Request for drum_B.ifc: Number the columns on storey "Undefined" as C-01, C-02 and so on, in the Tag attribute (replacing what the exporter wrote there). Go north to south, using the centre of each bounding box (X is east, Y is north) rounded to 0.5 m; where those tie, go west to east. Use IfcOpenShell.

First a look at what the model holds.

```python
import ifcopenshell
import ifcopenshell.util.element
import ifcopenshell.util.placement

model = ifcopenshell.open("drum_B.ifc")
print(model.schema)
storey = next(s for s in model.by_type("IfcBuildingStorey") if s.Name == "Undefined")
columns = [e for e in ifcopenshell.util.element.get_decomposition(storey) if e.is_a("IfcColumn")]
for e in sorted(columns, key=lambda e: e.id()):
    origin = ifcopenshell.util.placement.get_local_placement(e.ObjectPlacement)[:3, 3]
    print(e.id(), e.Tag, e.Name, origin.round(2) + 0.0, sep=" | ")
```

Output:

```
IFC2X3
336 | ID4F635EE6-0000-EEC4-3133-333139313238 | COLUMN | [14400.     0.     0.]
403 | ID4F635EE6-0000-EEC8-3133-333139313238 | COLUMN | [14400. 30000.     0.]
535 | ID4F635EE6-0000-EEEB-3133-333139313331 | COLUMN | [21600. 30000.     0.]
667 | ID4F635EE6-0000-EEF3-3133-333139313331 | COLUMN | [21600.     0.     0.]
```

```python
import ifcopenshell
import ifcopenshell.geom
import ifcopenshell.util.element
import ifcopenshell.util.shape

model = ifcopenshell.open("drum_B.ifc")
settings = ifcopenshell.geom.settings()
settings.set("use-world-coords", True)


def centre(element):
    shape = ifcopenshell.geom.create_shape(settings, element)
    return ifcopenshell.util.shape.get_bbox_centroid(shape.geometry)


storey = next(s for s in model.by_type("IfcBuildingStorey") if s.Name == "Undefined")
columns = [e for e in ifcopenshell.util.element.get_decomposition(storey) if e.is_a("IfcColumn")]

# Insertion points can sit at a corner or the storey origin, so sort by the geometry (in metres).
centres = {e: centre(e) for e in columns}
columns.sort(key=lambda e: (-round(centres[e][1] / 0.5), centres[e][0]))

for i, e in enumerate(columns, start=1):
    number = f"C-{i:02d}"
    e.Tag = number
    print(e.id(), number)

model.write("drum_B_rev.ifc")
```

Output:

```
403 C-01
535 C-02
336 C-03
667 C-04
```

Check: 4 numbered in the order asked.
